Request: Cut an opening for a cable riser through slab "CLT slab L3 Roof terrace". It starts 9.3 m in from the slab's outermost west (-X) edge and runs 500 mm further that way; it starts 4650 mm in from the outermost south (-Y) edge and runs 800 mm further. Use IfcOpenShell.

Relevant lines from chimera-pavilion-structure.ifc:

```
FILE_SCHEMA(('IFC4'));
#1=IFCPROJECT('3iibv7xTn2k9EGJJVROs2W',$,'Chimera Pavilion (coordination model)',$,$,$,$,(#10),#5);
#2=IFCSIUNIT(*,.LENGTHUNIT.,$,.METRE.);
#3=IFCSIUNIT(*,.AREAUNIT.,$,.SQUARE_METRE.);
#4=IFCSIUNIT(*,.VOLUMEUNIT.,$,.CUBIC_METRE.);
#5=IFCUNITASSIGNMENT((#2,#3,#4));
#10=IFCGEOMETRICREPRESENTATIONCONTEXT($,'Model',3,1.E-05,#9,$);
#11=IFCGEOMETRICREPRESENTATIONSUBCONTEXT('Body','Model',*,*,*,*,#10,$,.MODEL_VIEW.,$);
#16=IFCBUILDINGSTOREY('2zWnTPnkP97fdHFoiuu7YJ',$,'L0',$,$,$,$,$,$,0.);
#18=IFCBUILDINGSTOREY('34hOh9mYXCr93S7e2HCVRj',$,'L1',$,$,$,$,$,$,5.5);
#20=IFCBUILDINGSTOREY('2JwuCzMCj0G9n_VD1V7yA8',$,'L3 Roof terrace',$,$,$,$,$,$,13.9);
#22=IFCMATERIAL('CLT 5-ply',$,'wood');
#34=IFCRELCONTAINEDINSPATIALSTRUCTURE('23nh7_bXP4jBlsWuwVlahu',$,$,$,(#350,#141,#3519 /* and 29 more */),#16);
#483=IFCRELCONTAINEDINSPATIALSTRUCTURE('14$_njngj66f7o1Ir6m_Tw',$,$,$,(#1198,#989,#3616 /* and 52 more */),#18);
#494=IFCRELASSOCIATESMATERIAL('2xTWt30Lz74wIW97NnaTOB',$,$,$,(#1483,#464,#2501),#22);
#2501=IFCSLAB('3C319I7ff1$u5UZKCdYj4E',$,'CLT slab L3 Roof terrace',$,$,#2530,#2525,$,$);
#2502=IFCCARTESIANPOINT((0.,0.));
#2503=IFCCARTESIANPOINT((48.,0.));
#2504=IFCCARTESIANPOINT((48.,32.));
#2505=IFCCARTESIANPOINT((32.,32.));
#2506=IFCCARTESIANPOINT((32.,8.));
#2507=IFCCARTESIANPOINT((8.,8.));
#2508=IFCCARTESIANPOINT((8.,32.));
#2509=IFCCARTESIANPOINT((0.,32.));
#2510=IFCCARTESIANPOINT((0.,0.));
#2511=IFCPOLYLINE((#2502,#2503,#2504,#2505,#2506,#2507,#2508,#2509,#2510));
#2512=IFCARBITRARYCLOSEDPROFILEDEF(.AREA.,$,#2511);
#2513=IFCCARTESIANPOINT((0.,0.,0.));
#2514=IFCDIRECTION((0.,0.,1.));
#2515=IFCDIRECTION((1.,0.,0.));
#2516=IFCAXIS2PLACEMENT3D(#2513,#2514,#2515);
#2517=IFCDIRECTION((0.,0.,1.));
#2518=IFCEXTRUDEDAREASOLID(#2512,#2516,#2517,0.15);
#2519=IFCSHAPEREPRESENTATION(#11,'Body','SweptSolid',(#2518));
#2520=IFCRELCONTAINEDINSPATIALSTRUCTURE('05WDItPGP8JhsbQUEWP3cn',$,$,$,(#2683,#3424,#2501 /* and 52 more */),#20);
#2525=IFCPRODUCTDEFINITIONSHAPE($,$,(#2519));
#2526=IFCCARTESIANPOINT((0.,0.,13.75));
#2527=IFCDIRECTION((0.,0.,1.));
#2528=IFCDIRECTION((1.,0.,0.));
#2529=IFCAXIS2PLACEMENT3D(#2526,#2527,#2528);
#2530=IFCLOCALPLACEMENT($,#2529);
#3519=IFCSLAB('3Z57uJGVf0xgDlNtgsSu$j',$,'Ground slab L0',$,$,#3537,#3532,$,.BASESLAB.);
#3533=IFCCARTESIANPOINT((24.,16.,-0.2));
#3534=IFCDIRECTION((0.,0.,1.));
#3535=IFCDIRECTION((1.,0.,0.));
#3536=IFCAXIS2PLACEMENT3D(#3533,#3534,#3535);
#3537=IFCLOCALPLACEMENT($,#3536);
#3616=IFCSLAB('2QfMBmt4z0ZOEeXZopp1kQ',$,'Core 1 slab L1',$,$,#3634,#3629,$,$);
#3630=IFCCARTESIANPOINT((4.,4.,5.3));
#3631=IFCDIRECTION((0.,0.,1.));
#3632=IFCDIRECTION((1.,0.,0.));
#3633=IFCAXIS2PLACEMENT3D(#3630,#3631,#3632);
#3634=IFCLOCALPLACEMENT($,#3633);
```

```python
import numpy as np
import ifcopenshell
import ifcopenshell.api.feature
import ifcopenshell.api.geometry
import ifcopenshell.api.root
import ifcopenshell.geom
import ifcopenshell.util.placement
import ifcopenshell.util.representation
import ifcopenshell.util.shape
import ifcopenshell.util.unit

model = ifcopenshell.open("chimera-pavilion-structure.ifc")
unit_scale = ifcopenshell.util.unit.calculate_unit_scale(model)
settings = ifcopenshell.geom.settings()


def volume(element):
    """Net volume in cubic metres, openings subtracted."""
    shape = ifcopenshell.geom.create_shape(settings, element)
    return ifcopenshell.util.shape.get_volume(shape.geometry)


slab = model.by_id(2501)
before = volume(slab)

# Extent in the slab's own axes, in metres. The edges named are its -X and -Y sides.
slab_shape = ifcopenshell.geom.create_shape(settings, slab)
vertices = ifcopenshell.util.shape.get_vertices(slab_shape.geometry)
x_min, y_min, bottom = vertices.min(axis=0)
top = vertices[:, 2].max()

opening = ifcopenshell.api.root.create_entity(model, ifc_class="IfcOpeningElement", name="Cable riser opening", predefined_type="OPENING")
context = ifcopenshell.util.representation.get_context(model, "Model", "Body", "MODEL_VIEW")
width, depth = 0.5, 0.8
outline = [(0.0, 0.0), (width, 0.0), (width, depth), (0.0, depth), (0.0, 0.0)]
# Overshoot both faces by 50 mm so the cut is clean.
shape = ifcopenshell.api.geometry.add_slab_representation(
    model, context=context, depth=top - bottom + 0.1, polyline=outline
)
ifcopenshell.api.geometry.assign_representation(model, product=opening, representation=shape)

matrix = ifcopenshell.util.placement.get_local_placement(slab.ObjectPlacement)
matrix[:, 3] = matrix @ np.append(np.array([x_min + 9.3, y_min + 4.65, bottom - 0.05]) / unit_scale, 1.0)
ifcopenshell.api.geometry.edit_object_placement(model, product=opening, matrix=matrix, is_si=False)
ifcopenshell.api.feature.add_feature(model, feature=opening, element=slab)

after = volume(slab)

print(f"slab volume {before:.3f} -> {after:.3f} m3")

model.write("chimera-pavilion-structure-out.ifc")
```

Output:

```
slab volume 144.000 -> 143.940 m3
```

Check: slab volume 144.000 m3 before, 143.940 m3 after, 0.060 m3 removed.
